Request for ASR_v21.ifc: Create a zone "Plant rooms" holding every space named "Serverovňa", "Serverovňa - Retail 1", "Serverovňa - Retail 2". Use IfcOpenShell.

First a look at what the model holds.

```python
import ifcopenshell

model = ifcopenshell.open("ASR_v21.ifc")
print(model.schema)
seen = {}
for space in model.by_type("IfcSpace"):
    seen[space.LongName] = seen.get(space.LongName, 0) + 1
for name, count in sorted(seen.items(), key=str):
    print(count, "x", name)
print("zones:", [z.Name for z in model.by_type("IfcZone")][:20])
```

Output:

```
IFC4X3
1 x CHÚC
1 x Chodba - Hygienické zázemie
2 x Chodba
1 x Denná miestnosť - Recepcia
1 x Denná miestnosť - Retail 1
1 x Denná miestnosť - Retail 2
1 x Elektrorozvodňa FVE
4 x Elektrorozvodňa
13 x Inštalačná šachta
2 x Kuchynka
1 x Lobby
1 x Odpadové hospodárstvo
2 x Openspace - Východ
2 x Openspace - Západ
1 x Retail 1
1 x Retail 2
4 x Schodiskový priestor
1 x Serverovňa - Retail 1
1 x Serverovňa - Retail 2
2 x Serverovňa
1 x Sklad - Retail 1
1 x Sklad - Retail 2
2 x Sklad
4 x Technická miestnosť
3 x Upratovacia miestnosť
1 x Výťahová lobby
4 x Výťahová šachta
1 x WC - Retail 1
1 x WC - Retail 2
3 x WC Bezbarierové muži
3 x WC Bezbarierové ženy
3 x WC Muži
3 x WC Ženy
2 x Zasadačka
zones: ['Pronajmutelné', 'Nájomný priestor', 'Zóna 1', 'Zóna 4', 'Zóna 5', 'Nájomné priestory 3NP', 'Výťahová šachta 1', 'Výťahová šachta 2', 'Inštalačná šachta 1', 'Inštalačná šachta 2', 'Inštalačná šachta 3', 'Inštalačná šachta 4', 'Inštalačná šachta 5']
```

```python
import ifcopenshell
import ifcopenshell.api.group
import ifcopenshell.api.root

model = ifcopenshell.open("ASR_v21.ifc")

names = {"Serverovňa", "Serverovňa - Retail 1", "Serverovňa - Retail 2"}
spaces = [s for s in model.by_type("IfcSpace") if s.LongName in names]

zone = ifcopenshell.api.root.create_entity(model, ifc_class="IfcZone", name="Plant rooms")
ifcopenshell.api.group.assign_group(model, products=spaces, group=zone)
print(len(spaces), "spaces in", zone.Name)

model.write("ASR_v21_rev.ifc")
```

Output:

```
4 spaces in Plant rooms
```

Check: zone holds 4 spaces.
